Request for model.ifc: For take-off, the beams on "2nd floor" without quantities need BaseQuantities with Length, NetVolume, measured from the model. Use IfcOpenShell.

First a look at what the model holds.

```python
import ifcopenshell
import ifcopenshell.util.element
import ifcopenshell.util.unit

model = ifcopenshell.open("model.ifc")
print(model.schema)
for unit_type in ("LENGTHUNIT", "AREAUNIT", "VOLUMEUNIT"):
    print(unit_type, ifcopenshell.util.unit.calculate_unit_scale(model, unit_type))
storey = next(s for s in model.by_type("IfcBuildingStorey") if s.Name == "2nd floor")
beams = [e for e in ifcopenshell.util.element.get_decomposition(storey) if e.is_a("IfcBeam")]
for e in sorted(beams, key=lambda e: e.id()):
    print(e.id(), e.is_a(), e.Name, list(ifcopenshell.util.element.get_psets(e, qtos_only=True)), sep=" | ")
```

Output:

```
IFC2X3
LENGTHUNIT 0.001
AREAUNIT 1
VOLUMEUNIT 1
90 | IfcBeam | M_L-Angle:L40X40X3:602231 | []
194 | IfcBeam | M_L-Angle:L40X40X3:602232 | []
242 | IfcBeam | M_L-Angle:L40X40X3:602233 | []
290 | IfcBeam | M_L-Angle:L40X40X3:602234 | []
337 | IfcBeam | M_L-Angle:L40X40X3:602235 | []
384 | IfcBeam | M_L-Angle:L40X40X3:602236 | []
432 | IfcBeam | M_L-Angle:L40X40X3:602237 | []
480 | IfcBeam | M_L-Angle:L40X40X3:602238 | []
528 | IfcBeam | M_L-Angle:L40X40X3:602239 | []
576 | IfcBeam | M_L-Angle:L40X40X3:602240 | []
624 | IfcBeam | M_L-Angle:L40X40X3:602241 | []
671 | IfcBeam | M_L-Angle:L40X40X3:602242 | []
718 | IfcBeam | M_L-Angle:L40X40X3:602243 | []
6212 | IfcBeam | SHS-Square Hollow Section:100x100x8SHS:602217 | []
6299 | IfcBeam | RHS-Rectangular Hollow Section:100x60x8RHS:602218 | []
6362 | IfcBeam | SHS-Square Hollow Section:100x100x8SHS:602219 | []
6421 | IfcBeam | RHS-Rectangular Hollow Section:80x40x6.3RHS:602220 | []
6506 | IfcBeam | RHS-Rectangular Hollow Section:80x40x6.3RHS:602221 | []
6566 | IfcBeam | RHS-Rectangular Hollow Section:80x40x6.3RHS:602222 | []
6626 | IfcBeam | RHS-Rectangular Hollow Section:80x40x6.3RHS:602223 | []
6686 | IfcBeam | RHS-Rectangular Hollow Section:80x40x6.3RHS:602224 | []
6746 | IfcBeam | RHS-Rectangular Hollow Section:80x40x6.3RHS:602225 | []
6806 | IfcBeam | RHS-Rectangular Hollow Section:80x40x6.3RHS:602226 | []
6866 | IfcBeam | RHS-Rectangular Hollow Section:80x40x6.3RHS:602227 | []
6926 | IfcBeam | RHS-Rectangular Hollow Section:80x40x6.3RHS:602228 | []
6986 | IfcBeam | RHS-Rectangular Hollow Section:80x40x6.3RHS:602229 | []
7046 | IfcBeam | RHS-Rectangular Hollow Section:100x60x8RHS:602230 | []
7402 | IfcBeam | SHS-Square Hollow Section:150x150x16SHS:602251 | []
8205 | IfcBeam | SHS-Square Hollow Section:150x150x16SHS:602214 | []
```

```python
import ifcopenshell
import ifcopenshell.api.pset
import ifcopenshell.geom
import ifcopenshell.util.element
import ifcopenshell.util.shape
import ifcopenshell.util.unit

model = ifcopenshell.open("model.ifc")
unit_scale = ifcopenshell.util.unit.calculate_unit_scale(model)
volume_scale = ifcopenshell.util.unit.calculate_unit_scale(model, "VOLUMEUNIT")
settings = ifcopenshell.geom.settings()

storey = next(s for s in model.by_type("IfcBuildingStorey") if s.Name == "2nd floor")
beams = [e for e in ifcopenshell.util.element.get_decomposition(storey) if e.is_a("IfcBeam")]

for e in sorted(beams, key=lambda e: e.id()):
    if ifcopenshell.util.element.get_psets(e, qtos_only=True, should_inherit=False):
        continue
    # Geometry comes back in metres, in the element's own axes.
    shape = ifcopenshell.geom.create_shape(settings, e)
    values = {
        "Length": ifcopenshell.util.shape.get_max_xyz(shape.geometry) / unit_scale,
        "NetVolume": ifcopenshell.util.shape.get_volume(shape.geometry) / volume_scale,
    }
    qto = ifcopenshell.api.pset.add_qto(model, product=e, name="BaseQuantities")
    ifcopenshell.api.pset.edit_qto(model, qto=qto, properties=values)
    print(e.id(), {k: round(v, 3) for k, v in values.items()})

model.write("model_edited.ifc")
```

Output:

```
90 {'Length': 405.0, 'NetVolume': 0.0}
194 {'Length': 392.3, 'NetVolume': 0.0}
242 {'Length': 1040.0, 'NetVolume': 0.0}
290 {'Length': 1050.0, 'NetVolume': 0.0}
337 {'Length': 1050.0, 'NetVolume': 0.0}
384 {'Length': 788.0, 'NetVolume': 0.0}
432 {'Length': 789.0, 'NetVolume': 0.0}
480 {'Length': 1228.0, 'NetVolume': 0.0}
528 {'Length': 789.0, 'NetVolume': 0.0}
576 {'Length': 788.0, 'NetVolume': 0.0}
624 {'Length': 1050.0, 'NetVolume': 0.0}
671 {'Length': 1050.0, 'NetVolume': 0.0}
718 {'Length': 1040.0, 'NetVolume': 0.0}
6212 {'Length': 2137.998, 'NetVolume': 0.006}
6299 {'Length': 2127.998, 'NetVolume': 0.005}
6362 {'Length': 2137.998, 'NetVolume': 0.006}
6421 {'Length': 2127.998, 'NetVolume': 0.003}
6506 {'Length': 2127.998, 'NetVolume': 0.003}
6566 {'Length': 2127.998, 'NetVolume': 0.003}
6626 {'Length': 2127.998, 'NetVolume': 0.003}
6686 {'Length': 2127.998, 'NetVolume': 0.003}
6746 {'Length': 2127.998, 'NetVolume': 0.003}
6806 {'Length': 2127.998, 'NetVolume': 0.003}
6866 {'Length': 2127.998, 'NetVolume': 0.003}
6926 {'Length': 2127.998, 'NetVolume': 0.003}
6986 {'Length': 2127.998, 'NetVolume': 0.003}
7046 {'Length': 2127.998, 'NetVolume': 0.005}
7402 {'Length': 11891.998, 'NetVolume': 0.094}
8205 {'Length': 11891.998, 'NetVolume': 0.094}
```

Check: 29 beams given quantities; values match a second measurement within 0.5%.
